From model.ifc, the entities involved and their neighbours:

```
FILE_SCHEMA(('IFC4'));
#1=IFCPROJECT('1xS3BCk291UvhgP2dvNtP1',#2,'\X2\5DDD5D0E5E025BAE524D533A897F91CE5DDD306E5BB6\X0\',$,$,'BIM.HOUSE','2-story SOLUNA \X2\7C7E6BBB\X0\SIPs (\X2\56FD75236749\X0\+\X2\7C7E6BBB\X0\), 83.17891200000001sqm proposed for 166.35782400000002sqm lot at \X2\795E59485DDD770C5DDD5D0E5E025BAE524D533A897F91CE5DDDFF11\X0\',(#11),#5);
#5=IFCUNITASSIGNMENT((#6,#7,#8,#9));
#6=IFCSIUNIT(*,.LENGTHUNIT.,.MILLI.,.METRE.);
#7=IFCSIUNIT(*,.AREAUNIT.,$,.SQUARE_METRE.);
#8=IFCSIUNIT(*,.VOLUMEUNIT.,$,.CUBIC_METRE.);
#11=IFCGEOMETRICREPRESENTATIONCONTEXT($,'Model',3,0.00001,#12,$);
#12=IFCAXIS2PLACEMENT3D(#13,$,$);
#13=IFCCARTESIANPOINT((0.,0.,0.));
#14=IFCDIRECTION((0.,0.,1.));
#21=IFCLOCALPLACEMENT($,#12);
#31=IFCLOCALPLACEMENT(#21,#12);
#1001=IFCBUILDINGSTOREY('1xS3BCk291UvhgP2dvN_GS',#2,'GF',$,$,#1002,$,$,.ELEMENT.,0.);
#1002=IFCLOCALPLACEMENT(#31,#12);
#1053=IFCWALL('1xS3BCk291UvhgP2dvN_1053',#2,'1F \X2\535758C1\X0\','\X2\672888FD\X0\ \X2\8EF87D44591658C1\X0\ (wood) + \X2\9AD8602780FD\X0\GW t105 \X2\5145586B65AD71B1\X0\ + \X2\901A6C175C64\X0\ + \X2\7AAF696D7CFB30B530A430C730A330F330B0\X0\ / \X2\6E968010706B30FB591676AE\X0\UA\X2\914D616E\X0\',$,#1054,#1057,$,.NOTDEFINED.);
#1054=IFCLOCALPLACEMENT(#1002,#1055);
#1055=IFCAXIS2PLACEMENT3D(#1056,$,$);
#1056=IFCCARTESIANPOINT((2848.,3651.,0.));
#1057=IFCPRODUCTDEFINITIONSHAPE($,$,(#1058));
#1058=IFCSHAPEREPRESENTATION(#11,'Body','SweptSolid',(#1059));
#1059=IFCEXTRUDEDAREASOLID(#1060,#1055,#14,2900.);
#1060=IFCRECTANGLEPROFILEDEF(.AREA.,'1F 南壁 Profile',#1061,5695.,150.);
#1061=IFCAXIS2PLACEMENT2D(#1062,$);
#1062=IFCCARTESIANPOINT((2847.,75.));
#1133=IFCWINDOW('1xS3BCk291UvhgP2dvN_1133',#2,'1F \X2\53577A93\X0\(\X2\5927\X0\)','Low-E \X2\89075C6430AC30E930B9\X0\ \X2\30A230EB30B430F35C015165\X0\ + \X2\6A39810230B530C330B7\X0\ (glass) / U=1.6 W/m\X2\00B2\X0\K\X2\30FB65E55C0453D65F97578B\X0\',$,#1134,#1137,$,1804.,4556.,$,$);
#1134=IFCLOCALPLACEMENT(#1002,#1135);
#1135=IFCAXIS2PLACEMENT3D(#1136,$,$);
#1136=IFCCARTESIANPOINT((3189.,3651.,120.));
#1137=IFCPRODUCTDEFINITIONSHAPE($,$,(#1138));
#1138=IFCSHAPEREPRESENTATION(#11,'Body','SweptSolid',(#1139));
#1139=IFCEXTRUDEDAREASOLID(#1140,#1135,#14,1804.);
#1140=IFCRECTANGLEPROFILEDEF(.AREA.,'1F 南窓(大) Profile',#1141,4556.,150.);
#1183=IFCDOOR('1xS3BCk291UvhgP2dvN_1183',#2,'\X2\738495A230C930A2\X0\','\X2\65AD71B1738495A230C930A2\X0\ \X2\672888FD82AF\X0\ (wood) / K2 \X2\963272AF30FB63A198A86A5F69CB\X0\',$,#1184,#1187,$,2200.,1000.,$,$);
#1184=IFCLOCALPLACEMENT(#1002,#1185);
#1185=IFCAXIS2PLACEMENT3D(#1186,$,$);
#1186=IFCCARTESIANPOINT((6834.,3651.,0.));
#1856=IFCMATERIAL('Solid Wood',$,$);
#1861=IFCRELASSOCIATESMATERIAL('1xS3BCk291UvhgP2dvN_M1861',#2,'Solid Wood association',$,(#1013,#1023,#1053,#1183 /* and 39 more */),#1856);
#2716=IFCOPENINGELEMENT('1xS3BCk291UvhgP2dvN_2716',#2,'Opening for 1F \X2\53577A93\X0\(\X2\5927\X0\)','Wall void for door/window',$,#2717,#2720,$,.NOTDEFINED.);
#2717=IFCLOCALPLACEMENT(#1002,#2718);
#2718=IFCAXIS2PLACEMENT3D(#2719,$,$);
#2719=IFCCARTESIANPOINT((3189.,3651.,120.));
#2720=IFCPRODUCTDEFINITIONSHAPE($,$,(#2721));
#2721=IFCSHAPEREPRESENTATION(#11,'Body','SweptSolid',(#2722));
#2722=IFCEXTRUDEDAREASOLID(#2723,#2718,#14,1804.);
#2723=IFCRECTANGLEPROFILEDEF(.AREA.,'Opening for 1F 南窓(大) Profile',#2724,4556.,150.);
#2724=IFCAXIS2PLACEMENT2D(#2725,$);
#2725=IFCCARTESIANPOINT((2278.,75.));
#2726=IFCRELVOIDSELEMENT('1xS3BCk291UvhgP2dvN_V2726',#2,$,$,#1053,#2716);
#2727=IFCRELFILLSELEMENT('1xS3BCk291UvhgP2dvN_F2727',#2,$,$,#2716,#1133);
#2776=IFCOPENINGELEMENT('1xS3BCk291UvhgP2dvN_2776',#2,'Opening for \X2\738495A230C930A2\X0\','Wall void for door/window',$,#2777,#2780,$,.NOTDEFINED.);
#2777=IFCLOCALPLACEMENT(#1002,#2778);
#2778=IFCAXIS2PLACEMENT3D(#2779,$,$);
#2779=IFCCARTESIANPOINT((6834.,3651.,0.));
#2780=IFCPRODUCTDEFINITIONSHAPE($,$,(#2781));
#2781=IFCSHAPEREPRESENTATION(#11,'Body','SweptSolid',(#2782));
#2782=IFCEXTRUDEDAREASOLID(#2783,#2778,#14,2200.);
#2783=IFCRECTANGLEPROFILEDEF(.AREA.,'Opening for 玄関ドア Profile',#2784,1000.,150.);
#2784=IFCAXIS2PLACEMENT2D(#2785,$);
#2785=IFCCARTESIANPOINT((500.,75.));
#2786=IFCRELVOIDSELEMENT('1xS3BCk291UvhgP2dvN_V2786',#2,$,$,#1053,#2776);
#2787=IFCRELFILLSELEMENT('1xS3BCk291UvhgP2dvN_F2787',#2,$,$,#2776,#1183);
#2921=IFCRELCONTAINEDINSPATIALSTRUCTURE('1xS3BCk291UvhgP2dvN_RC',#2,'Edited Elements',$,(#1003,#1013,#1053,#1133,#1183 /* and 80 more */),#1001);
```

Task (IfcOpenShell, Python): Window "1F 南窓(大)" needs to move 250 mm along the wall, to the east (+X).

```python
import ifcopenshell
import ifcopenshell.api.geometry
import ifcopenshell.util.placement
import ifcopenshell.util.unit

model = ifcopenshell.open("model.ifc")
unit_scale = ifcopenshell.util.unit.calculate_unit_scale(model)

window = model.by_guid("1xS3BCk291UvhgP2dvN_1133")
opening = window.FillsVoids[0].RelatingOpeningElement
wall = opening.VoidsElements[0].RelatingBuildingElement

wall_matrix = ifcopenshell.util.placement.get_local_placement(wall.ObjectPlacement)
shift = wall_matrix[:3, 0] * 0.25 / unit_scale
before = ifcopenshell.util.placement.get_local_placement(window.ObjectPlacement)[:3, 3].copy()

# The window is not placed relative to its opening, so move both.
for product in (opening, window):
    matrix = ifcopenshell.util.placement.get_local_placement(product.ObjectPlacement)
    matrix[:3, 3] += shift
    ifcopenshell.api.geometry.edit_object_placement(model, product=product, matrix=matrix, is_si=False)

after = ifcopenshell.util.placement.get_local_placement(window.ObjectPlacement)[:3, 3]
print("window moved by", (after - before).round(3) + 0.0)

model.write("model-out.ifc")
```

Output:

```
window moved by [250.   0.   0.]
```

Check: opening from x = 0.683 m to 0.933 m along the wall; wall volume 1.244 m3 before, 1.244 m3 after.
